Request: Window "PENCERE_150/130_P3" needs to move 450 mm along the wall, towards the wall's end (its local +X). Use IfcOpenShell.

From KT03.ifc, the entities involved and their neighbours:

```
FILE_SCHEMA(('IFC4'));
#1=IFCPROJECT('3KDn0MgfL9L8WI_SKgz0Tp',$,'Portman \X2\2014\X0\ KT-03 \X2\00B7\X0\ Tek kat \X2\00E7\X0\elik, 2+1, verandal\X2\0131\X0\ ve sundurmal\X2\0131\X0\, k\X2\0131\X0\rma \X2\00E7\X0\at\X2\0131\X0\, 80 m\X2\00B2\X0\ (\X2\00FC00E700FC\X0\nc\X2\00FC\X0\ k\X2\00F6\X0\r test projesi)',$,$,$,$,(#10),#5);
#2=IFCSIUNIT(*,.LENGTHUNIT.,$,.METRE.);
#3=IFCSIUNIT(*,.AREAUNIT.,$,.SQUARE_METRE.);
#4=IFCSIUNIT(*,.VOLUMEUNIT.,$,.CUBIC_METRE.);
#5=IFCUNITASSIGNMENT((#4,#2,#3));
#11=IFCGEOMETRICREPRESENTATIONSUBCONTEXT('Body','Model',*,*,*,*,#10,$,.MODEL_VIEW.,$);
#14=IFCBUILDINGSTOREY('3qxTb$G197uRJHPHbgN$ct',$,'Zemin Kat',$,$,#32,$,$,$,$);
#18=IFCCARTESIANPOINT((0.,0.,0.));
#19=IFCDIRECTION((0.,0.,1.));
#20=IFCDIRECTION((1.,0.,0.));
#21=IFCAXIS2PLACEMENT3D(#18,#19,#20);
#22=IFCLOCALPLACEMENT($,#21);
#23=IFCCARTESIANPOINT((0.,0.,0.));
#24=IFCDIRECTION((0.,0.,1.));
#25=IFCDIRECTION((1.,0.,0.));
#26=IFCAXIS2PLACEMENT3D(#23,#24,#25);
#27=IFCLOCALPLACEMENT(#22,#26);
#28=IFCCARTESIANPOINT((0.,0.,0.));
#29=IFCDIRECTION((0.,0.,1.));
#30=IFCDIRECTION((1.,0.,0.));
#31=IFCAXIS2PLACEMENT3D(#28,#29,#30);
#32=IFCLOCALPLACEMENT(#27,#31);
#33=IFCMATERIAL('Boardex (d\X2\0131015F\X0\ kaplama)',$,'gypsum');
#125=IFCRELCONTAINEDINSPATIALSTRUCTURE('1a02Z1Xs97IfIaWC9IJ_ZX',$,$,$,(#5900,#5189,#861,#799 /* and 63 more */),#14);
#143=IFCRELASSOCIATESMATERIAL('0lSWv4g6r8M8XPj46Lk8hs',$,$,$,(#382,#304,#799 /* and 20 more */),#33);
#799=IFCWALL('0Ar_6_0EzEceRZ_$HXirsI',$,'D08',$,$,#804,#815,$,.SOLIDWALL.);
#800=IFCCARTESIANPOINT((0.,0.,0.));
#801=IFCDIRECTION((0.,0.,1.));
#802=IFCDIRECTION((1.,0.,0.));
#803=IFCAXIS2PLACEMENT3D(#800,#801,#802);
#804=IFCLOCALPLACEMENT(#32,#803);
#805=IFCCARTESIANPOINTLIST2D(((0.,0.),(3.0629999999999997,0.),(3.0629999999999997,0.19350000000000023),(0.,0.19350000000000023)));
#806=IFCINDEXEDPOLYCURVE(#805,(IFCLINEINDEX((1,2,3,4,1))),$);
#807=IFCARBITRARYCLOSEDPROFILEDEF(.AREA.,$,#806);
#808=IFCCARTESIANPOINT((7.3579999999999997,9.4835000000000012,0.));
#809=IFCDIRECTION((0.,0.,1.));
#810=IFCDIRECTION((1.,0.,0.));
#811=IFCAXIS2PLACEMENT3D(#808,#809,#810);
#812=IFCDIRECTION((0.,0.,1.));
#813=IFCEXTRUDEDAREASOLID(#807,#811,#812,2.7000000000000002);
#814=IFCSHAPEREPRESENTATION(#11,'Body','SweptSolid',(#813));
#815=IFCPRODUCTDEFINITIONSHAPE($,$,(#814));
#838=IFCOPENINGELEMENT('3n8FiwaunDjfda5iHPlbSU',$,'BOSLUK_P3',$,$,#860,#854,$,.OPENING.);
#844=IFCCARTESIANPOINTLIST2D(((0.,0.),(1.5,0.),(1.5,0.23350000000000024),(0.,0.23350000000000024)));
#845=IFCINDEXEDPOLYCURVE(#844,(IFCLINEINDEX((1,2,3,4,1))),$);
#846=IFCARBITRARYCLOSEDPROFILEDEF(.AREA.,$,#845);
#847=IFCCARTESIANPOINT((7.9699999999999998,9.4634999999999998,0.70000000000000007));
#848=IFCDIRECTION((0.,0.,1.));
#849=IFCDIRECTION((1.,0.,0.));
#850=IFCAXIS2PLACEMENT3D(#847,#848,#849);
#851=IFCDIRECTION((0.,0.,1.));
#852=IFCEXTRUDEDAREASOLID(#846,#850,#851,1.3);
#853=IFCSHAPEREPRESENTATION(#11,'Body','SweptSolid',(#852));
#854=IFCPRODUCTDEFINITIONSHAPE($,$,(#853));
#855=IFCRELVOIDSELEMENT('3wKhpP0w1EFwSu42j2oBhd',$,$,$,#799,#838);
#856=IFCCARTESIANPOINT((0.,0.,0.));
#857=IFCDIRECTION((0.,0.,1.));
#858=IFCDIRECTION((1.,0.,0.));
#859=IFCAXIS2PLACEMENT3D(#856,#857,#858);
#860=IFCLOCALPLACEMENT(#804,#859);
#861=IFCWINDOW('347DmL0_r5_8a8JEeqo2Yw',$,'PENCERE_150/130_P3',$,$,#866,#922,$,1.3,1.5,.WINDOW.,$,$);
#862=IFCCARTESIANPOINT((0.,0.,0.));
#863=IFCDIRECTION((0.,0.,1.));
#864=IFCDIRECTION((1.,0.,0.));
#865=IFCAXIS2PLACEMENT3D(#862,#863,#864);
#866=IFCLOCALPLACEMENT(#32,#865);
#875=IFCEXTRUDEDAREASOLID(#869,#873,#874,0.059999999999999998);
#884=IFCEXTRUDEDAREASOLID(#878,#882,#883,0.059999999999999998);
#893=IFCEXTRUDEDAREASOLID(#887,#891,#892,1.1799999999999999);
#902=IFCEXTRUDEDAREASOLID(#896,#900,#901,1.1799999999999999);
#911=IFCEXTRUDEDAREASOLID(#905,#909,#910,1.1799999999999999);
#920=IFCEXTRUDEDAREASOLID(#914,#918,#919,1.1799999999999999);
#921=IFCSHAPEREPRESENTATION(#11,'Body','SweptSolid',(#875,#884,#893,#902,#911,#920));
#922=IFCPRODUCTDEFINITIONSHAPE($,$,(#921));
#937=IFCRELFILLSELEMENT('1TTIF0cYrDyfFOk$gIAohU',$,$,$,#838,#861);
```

```python
import ifcopenshell
import ifcopenshell.api.geometry
import ifcopenshell.util.placement
import ifcopenshell.util.unit

model = ifcopenshell.open("KT03.ifc")
unit_scale = ifcopenshell.util.unit.calculate_unit_scale(model)

window = model.by_id(861)
opening = window.FillsVoids[0].RelatingOpeningElement
wall = opening.VoidsElements[0].RelatingBuildingElement

wall_matrix = ifcopenshell.util.placement.get_local_placement(wall.ObjectPlacement)
shift = wall_matrix[:3, 0] * 0.45 / unit_scale
before = ifcopenshell.util.placement.get_local_placement(window.ObjectPlacement)[:3, 3].copy()

# The window is not placed relative to its opening, so move both.
for product in (opening, window):
    matrix = ifcopenshell.util.placement.get_local_placement(product.ObjectPlacement)
    matrix[:3, 3] += shift
    ifcopenshell.api.geometry.edit_object_placement(model, product=product, matrix=matrix, is_si=False)

after = ifcopenshell.util.placement.get_local_placement(window.ObjectPlacement)[:3, 3]
print("window moved by", (after - before).round(3) + 0.0)

model.write("KT03-out.ifc")
```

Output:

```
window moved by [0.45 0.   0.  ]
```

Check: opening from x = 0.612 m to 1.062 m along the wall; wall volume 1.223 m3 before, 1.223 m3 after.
